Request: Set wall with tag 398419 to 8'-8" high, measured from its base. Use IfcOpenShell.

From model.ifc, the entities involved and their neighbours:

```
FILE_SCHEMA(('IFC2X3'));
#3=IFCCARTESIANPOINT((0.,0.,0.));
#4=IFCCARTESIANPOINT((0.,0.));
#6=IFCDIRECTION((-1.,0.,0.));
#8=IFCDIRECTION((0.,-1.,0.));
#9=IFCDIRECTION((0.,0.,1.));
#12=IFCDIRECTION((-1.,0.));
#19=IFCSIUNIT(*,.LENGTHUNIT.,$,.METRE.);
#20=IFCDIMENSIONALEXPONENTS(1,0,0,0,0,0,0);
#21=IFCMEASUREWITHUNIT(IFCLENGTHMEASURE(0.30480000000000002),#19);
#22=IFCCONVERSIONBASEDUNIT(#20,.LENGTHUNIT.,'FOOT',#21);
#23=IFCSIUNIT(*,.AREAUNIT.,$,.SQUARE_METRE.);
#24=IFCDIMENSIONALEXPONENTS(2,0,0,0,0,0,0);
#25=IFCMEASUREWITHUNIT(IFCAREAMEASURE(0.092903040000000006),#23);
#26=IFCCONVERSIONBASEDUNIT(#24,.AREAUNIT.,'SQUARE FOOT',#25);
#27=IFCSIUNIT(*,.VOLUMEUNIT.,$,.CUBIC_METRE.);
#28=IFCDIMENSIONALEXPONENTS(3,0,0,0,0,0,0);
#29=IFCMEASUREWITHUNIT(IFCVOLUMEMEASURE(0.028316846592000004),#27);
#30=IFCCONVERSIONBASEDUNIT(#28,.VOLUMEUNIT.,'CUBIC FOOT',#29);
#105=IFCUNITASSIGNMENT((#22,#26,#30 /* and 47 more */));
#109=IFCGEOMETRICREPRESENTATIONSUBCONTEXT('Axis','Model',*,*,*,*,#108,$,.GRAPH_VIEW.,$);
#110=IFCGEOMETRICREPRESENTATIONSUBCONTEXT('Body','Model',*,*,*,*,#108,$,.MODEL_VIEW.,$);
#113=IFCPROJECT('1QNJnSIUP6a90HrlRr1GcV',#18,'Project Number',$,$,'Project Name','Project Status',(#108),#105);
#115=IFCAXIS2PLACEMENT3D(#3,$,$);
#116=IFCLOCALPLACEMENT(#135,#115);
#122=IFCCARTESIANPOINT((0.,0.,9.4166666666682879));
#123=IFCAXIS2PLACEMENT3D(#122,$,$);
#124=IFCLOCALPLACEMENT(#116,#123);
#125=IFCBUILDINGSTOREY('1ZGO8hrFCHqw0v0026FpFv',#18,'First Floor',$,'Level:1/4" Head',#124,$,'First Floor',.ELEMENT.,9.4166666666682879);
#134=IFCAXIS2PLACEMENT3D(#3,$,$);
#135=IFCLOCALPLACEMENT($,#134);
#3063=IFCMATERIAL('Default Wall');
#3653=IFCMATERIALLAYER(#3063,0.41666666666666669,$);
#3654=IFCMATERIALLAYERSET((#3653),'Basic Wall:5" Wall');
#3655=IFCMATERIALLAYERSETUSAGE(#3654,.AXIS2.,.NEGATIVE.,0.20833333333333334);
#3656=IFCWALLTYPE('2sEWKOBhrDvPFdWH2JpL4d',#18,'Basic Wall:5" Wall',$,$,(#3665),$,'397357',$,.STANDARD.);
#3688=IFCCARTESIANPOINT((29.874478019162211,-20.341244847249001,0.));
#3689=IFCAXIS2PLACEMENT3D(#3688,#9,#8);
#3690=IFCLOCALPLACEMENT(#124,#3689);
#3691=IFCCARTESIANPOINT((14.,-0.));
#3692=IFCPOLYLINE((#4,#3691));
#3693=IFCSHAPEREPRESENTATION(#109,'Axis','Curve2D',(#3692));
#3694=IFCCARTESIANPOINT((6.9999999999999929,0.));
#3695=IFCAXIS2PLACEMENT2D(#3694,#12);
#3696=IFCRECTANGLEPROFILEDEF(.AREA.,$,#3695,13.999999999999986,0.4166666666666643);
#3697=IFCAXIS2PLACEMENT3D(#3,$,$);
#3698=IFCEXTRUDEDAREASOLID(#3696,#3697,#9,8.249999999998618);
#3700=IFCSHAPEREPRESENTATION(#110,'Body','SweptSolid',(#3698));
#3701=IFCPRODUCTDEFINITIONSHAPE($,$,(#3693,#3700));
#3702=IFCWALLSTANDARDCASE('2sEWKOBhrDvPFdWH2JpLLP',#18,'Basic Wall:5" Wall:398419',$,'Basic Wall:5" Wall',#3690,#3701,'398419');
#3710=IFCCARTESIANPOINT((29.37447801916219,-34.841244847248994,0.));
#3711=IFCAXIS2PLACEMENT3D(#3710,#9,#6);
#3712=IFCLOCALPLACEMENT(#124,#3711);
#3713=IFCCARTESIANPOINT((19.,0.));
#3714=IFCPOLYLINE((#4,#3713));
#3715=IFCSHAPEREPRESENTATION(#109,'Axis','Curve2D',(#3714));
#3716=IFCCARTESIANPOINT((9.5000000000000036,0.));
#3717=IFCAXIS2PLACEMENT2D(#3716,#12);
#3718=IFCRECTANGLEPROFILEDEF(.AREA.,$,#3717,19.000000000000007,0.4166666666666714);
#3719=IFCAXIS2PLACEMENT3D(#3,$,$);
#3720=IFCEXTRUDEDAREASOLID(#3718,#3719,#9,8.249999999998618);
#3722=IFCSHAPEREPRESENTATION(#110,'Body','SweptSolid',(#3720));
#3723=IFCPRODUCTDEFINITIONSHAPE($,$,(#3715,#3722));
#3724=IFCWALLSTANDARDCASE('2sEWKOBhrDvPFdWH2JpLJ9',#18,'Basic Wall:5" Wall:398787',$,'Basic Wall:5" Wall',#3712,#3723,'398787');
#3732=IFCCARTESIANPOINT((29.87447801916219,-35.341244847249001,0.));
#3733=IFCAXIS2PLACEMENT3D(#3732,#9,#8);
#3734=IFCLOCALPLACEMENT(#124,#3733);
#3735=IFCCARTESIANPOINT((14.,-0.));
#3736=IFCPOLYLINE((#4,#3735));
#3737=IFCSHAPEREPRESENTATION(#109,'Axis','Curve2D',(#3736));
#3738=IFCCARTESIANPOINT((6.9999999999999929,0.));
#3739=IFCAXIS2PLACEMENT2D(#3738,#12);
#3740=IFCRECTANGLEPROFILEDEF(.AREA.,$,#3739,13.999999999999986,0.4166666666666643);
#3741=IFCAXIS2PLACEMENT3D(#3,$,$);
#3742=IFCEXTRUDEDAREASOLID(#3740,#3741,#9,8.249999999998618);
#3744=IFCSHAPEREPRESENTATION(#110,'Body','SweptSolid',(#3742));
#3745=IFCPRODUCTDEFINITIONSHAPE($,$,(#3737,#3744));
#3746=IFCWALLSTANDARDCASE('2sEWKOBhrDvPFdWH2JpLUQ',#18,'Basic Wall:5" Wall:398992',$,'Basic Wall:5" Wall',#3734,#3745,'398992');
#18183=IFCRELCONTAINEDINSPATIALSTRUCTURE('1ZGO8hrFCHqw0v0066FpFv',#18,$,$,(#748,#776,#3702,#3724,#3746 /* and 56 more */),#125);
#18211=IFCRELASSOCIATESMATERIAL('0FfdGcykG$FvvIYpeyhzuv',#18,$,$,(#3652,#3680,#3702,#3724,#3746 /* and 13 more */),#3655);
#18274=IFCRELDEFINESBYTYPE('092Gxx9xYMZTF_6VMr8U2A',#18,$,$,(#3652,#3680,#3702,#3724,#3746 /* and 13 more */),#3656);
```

```python
import ifcopenshell
import ifcopenshell.geom
import ifcopenshell.util.representation
import ifcopenshell.util.shape
import ifcopenshell.util.unit

model = ifcopenshell.open("model.ifc")
unit_scale = ifcopenshell.util.unit.calculate_unit_scale(model)
settings = ifcopenshell.geom.settings()


def volume(element):
    """Net volume in cubic metres, openings subtracted."""
    shape = ifcopenshell.geom.create_shape(settings, element)
    return ifcopenshell.util.shape.get_volume(shape.geometry)


wall = model.by_id(3702)
before = volume(wall)

body = ifcopenshell.util.representation.get_representation(wall, "Model", "Body")
solid = body.Items[0]
old_height = solid.Depth
solid.Depth = 104 * 0.0254 / unit_scale
after = volume(wall)

print(f"height {old_height:g} -> {solid.Depth:g}, volume {before:.3f} -> {after:.3f} m3")

model.write("model_rev.ifc")
```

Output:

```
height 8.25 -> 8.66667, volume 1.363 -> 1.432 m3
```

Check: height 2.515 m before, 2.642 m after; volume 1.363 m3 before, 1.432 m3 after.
